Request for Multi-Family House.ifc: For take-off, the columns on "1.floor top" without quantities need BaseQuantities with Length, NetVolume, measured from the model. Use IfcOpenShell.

First a look at what the model holds.

```python
import ifcopenshell
import ifcopenshell.util.element
import ifcopenshell.util.unit

model = ifcopenshell.open("Multi-Family House.ifc")
print(model.schema)
for unit_type in ("LENGTHUNIT", "AREAUNIT", "VOLUMEUNIT"):
    print(unit_type, ifcopenshell.util.unit.calculate_unit_scale(model, unit_type))
storey = next(s for s in model.by_type("IfcBuildingStorey") if s.Name == "1.floor top")
columns = [e for e in ifcopenshell.util.element.get_decomposition(storey) if e.is_a("IfcColumn")]
for e in sorted(columns, key=lambda e: e.id()):
    print(e.id(), e.is_a(), e.Name, list(ifcopenshell.util.element.get_psets(e, qtos_only=True)), sep=" | ")
```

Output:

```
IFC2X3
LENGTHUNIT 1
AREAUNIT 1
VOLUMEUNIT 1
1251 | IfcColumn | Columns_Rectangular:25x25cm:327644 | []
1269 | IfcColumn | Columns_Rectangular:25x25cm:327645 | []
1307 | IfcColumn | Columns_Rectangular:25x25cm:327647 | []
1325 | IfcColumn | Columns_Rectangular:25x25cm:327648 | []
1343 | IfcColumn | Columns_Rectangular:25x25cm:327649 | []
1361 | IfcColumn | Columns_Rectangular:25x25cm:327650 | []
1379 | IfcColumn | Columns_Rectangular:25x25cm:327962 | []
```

```python
import ifcopenshell
import ifcopenshell.api.pset
import ifcopenshell.geom
import ifcopenshell.util.element
import ifcopenshell.util.shape
import ifcopenshell.util.unit

model = ifcopenshell.open("Multi-Family House.ifc")
unit_scale = ifcopenshell.util.unit.calculate_unit_scale(model)
volume_scale = ifcopenshell.util.unit.calculate_unit_scale(model, "VOLUMEUNIT")
settings = ifcopenshell.geom.settings()

storey = next(s for s in model.by_type("IfcBuildingStorey") if s.Name == "1.floor top")
columns = [e for e in ifcopenshell.util.element.get_decomposition(storey) if e.is_a("IfcColumn")]

for e in sorted(columns, key=lambda e: e.id()):
    if ifcopenshell.util.element.get_psets(e, qtos_only=True, should_inherit=False):
        continue
    # Geometry comes back in metres, in the element's own axes.
    shape = ifcopenshell.geom.create_shape(settings, e)
    values = {
        "Length": ifcopenshell.util.shape.get_z(shape.geometry) / unit_scale,
        "NetVolume": ifcopenshell.util.shape.get_volume(shape.geometry) / volume_scale,
    }
    qto = ifcopenshell.api.pset.add_qto(model, product=e, name="BaseQuantities")
    ifcopenshell.api.pset.edit_qto(model, qto=qto, properties=values)
    print(e.id(), {k: round(v, 3) for k, v in values.items()})

model.write("Multi-Family House_v2.ifc")
```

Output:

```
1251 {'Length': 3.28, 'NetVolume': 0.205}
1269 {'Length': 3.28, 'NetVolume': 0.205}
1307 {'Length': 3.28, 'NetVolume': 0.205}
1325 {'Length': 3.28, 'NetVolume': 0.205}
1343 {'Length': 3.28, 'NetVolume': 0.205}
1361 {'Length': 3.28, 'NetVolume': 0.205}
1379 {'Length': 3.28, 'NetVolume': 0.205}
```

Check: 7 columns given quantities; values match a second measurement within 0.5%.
